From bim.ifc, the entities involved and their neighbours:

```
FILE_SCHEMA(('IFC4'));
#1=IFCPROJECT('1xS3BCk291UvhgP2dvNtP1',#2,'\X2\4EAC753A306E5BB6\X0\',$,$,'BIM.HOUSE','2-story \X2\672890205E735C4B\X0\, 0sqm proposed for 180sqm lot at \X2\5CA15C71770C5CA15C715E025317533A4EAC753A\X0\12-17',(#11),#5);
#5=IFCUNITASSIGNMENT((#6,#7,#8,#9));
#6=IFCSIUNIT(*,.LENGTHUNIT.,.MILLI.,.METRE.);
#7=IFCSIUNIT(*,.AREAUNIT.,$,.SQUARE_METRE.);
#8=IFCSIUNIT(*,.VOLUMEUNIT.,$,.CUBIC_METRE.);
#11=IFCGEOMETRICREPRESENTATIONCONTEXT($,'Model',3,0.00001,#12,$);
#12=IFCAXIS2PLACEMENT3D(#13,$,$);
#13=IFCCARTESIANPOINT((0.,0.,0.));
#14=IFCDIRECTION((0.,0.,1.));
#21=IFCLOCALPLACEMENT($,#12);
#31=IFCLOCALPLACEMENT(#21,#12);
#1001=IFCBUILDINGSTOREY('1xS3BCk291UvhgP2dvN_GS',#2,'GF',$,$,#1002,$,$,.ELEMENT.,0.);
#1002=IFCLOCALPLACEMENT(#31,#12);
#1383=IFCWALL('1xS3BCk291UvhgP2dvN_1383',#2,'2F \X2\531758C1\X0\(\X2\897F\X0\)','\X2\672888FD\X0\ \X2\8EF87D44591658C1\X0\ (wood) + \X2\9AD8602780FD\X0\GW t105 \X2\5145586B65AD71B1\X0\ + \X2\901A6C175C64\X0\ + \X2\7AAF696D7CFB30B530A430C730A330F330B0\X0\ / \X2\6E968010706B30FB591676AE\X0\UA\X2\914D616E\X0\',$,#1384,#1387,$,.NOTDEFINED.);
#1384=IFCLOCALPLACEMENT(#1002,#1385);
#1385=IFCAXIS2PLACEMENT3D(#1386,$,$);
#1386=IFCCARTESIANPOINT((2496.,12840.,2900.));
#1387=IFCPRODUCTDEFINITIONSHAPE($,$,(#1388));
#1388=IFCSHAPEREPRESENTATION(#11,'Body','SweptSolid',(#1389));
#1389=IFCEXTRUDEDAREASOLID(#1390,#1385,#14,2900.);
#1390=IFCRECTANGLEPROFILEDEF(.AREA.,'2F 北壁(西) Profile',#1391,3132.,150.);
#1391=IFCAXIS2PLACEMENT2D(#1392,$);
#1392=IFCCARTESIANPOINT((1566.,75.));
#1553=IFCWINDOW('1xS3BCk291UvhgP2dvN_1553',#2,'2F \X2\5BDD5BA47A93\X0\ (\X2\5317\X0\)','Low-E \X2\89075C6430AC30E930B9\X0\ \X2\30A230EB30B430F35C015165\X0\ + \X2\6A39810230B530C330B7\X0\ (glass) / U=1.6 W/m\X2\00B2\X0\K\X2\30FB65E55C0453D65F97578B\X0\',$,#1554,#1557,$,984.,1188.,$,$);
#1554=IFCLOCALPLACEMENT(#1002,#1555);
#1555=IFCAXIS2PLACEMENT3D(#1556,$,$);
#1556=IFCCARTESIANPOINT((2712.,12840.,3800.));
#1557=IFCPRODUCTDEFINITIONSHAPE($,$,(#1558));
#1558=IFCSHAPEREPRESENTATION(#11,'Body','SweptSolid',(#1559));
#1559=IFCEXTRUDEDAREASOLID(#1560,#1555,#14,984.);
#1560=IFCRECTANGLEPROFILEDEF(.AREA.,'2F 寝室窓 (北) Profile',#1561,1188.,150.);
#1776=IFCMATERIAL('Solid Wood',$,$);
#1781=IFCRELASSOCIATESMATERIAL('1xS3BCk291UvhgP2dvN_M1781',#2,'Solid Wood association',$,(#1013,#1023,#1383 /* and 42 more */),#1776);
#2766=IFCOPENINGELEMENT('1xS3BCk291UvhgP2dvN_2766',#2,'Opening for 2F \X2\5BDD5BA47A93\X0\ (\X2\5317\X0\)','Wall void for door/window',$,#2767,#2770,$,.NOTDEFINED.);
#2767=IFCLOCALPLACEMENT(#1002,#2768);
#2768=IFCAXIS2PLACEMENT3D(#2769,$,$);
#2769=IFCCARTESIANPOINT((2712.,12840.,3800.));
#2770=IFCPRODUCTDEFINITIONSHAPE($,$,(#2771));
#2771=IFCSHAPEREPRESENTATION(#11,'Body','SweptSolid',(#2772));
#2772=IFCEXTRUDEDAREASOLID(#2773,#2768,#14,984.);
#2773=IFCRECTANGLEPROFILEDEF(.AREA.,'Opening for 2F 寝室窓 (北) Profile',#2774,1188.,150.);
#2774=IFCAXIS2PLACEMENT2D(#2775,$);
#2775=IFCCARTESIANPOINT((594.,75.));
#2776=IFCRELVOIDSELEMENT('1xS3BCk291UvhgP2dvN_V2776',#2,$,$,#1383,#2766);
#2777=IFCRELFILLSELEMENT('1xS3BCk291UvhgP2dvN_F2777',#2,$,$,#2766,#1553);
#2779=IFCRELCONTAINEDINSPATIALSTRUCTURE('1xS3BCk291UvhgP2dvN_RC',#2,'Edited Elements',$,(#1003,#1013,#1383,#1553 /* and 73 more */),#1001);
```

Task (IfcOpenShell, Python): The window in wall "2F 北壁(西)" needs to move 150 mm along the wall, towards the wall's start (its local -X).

```python
import ifcopenshell
import ifcopenshell.api.geometry
import ifcopenshell.util.placement
import ifcopenshell.util.unit

model = ifcopenshell.open("bim.ifc")
unit_scale = ifcopenshell.util.unit.calculate_unit_scale(model)

window = model.by_guid("1xS3BCk291UvhgP2dvN_1553")
opening = window.FillsVoids[0].RelatingOpeningElement
wall = opening.VoidsElements[0].RelatingBuildingElement

wall_matrix = ifcopenshell.util.placement.get_local_placement(wall.ObjectPlacement)
shift = wall_matrix[:3, 0] * -0.15 / unit_scale
before = ifcopenshell.util.placement.get_local_placement(window.ObjectPlacement)[:3, 3].copy()

# The window is not placed relative to its opening, so move both.
for product in (opening, window):
    matrix = ifcopenshell.util.placement.get_local_placement(product.ObjectPlacement)
    matrix[:3, 3] += shift
    ifcopenshell.api.geometry.edit_object_placement(model, product=product, matrix=matrix, is_si=False)

after = ifcopenshell.util.placement.get_local_placement(window.ObjectPlacement)[:3, 3]
print("window moved by", (after - before).round(3) + 0.0)

model.write("bim_rev.ifc")
```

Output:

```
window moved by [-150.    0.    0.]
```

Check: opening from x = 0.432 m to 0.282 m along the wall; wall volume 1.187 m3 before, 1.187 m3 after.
